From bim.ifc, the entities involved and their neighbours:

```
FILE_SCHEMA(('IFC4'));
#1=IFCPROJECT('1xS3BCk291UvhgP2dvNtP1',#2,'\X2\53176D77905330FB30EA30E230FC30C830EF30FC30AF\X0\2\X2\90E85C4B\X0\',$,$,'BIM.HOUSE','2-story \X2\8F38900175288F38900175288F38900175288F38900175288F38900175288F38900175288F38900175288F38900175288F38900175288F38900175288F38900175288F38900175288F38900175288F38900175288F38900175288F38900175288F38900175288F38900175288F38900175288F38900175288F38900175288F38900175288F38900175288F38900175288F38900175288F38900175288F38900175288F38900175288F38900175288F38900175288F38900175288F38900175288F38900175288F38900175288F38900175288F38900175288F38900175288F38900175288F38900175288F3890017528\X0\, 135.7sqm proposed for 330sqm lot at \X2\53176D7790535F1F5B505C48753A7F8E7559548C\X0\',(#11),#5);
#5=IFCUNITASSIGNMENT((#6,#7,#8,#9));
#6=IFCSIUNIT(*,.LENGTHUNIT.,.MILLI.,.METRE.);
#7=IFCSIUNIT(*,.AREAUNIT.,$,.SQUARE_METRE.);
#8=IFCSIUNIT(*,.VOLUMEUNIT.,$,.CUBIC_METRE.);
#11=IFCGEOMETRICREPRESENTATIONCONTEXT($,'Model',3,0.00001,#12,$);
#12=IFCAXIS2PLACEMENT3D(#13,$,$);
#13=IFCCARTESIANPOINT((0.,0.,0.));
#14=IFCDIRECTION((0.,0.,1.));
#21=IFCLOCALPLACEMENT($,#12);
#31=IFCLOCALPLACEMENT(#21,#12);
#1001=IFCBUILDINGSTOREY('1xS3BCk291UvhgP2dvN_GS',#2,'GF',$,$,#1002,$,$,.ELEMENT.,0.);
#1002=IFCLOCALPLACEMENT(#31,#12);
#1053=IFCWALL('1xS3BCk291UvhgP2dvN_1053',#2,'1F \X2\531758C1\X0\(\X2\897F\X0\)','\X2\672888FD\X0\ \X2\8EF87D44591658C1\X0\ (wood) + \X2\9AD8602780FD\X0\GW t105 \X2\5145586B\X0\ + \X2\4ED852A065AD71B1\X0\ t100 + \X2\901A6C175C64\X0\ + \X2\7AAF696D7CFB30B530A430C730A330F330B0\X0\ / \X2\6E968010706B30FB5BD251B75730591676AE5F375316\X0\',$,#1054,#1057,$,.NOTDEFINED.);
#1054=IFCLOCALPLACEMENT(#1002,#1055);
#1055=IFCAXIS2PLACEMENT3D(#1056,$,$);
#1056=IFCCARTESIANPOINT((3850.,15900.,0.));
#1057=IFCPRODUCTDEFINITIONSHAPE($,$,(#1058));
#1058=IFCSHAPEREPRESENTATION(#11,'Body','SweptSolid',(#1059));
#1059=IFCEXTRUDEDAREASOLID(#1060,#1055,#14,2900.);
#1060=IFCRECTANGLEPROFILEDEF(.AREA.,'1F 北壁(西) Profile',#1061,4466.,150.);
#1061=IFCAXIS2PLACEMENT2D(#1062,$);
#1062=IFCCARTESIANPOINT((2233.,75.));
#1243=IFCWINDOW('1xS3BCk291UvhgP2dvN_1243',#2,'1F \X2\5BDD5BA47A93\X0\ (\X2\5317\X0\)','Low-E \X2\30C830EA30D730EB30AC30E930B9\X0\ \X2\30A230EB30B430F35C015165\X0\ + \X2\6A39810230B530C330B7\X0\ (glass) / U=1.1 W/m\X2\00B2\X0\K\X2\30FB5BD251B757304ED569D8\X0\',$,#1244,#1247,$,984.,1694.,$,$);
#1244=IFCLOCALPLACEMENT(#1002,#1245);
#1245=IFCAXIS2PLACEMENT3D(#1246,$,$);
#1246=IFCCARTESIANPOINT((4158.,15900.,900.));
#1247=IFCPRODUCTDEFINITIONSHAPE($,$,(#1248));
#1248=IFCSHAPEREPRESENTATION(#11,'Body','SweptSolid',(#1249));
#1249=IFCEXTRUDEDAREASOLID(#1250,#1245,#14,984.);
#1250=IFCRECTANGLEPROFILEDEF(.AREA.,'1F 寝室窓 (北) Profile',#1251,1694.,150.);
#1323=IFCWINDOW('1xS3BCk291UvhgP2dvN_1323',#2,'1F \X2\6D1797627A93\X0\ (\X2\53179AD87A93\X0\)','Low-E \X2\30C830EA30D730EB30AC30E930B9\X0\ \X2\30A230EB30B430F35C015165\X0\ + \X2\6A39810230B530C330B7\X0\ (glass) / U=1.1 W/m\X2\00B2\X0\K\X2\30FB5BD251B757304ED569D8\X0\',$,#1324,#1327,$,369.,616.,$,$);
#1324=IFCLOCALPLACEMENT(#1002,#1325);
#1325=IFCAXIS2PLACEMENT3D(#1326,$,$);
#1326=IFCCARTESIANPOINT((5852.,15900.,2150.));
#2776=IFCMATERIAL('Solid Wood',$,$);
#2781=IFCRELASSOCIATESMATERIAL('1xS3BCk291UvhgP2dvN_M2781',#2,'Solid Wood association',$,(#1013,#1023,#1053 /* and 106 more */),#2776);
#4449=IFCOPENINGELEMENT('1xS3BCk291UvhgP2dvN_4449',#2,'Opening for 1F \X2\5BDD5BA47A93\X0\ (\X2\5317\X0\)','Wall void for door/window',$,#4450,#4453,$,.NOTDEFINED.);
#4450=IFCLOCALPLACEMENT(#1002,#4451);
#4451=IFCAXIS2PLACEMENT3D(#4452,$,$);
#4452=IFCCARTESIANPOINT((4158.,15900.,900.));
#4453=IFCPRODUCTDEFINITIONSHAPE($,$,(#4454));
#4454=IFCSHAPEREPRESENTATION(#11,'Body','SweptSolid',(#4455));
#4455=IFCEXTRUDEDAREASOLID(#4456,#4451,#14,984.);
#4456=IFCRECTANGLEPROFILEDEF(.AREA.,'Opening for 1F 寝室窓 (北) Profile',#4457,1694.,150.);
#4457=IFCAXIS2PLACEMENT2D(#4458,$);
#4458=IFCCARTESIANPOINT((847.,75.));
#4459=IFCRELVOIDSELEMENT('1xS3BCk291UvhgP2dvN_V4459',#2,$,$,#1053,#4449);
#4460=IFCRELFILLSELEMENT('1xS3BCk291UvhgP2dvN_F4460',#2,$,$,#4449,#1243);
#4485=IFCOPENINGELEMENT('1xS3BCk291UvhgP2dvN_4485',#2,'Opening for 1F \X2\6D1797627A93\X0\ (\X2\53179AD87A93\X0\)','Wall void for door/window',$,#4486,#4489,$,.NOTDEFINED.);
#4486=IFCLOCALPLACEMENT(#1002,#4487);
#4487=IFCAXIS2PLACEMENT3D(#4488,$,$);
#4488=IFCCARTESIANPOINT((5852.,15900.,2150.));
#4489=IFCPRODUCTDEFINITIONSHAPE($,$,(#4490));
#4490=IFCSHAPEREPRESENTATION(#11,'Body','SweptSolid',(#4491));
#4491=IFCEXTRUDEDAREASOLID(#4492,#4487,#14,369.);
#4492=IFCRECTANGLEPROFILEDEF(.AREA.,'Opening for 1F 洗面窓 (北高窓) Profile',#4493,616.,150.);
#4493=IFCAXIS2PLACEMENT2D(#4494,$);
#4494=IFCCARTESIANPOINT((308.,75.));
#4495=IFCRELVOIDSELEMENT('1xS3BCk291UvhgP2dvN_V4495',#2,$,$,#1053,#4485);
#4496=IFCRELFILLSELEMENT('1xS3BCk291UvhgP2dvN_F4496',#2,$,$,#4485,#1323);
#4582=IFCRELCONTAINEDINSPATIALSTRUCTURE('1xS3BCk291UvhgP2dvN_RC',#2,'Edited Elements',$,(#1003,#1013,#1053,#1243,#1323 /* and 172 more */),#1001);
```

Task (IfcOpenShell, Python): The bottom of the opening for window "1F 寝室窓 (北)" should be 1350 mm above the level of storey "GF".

```python
import numpy as np
import ifcopenshell
import ifcopenshell.api.geometry
import ifcopenshell.geom
import ifcopenshell.util.element
import ifcopenshell.util.placement
import ifcopenshell.util.shape
import ifcopenshell.util.unit

model = ifcopenshell.open("bim.ifc")
unit_scale = ifcopenshell.util.unit.calculate_unit_scale(model)

window = model.by_guid("1xS3BCk291UvhgP2dvN_1243")
opening = window.FillsVoids[0].RelatingOpeningElement
storey = ifcopenshell.util.element.get_container(window, ifc_class="IfcBuildingStorey")
level = ifcopenshell.util.placement.get_local_placement(storey.ObjectPlacement)[2, 3]

# The opening's origin need not be at the sill, so measure its lowest point.
shape = ifcopenshell.geom.create_shape(ifcopenshell.geom.settings(), opening)
bottom = ifcopenshell.util.shape.get_shape_bottom_elevation(shape, shape.geometry) / unit_scale
dz = level + 1350.0 - bottom

shift = np.array([0.0, 0.0, dz])
# The window is not placed relative to its opening, so move both.
for product in (opening, window):
    matrix = ifcopenshell.util.placement.get_local_placement(product.ObjectPlacement)
    matrix[:3, 3] += shift
    ifcopenshell.api.geometry.edit_object_placement(model, product=product, matrix=matrix, is_si=False)

print(f"moved by {dz * unit_scale:+.3f} m")

model.write("bim_updated.ifc")
```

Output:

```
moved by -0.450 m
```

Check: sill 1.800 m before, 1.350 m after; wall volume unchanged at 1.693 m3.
